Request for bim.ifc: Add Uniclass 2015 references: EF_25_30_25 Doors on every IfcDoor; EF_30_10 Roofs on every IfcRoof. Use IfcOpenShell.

First a look at what the model holds.

```python
import ifcopenshell

model = ifcopenshell.open("bim.ifc")
print(model.schema)
print("classifications:", [c.Name for c in model.by_type("IfcClassification")])
for ifc_class in ("IfcDoor", "IfcRoof", "IfcStair", "IfcWall", "IfcWindow"):
    print(ifc_class, len(model.by_type(ifc_class)))
```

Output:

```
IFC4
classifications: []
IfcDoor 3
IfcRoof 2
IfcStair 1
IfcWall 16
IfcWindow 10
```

```python
import ifcopenshell
import ifcopenshell.api.classification

model = ifcopenshell.open("bim.ifc")

system = ifcopenshell.api.classification.add_classification(model, classification="Uniclass 2015")

codes = {
    "IfcDoor": ("EF_25_30_25", "Doors"),
    "IfcRoof": ("EF_30_10", "Roofs"),
}
for ifc_class, (code, name) in codes.items():
    products = model.by_type(ifc_class)
    ifcopenshell.api.classification.add_reference(
        model, products=products, classification=system, identification=code, name=name
    )
    print(code, len(products))

model.write("bim_updated.ifc")
```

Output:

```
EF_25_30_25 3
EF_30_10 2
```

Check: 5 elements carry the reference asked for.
